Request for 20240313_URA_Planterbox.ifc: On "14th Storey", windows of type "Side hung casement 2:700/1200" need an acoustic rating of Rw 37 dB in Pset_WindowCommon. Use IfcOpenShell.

First a look at what the model holds.

```python
import ifcopenshell
import ifcopenshell.util.element

model = ifcopenshell.open("20240313_URA_Planterbox.ifc")
print(model.schema)
storey = next(s for s in model.by_type("IfcBuildingStorey") if s.Name == "14th Storey")
windows = [e for e in ifcopenshell.util.element.get_decomposition(storey) if e.is_a("IfcWindow")]
seen = {}
for e in windows:
    element_type = ifcopenshell.util.element.get_type(e)
    key = (element_type.Name if element_type != e and element_type else None, ifcopenshell.util.element.get_pset(e, "Pset_WindowCommon", "AcousticRating"))
    seen[key] = seen.get(key, 0) + 1
for (name, value), count in sorted(seen.items(), key=str):
    print(count, "x", name, "|", value)
```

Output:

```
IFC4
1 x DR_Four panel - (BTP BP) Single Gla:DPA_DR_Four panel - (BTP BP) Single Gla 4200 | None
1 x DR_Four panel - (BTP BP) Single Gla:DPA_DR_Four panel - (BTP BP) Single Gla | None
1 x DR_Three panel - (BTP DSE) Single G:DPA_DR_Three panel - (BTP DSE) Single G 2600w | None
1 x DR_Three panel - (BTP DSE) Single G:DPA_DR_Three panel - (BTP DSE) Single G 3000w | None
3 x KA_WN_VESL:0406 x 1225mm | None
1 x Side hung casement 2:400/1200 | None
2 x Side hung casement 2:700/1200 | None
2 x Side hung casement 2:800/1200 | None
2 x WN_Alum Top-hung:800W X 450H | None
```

```python
import ifcopenshell
import ifcopenshell.api.pset
import ifcopenshell.util.element

model = ifcopenshell.open("20240313_URA_Planterbox.ifc")

storey = next(s for s in model.by_type("IfcBuildingStorey") if s.Name == "14th Storey")
windows = [e for e in ifcopenshell.util.element.get_decomposition(storey) if e.is_a("IfcWindow")]

count = 0
for e in windows:
    element_type = ifcopenshell.util.element.get_type(e)
    if element_type in (None, e) or element_type.Name != "Side hung casement 2:700/1200":
        continue
    # add_pset returns the element's existing set when there is one.
    pset = ifcopenshell.api.pset.add_pset(model, product=e, name="Pset_WindowCommon")
    ifcopenshell.api.pset.edit_pset(model, pset=pset, properties={"AcousticRating": "Rw 37 dB"})
    count += 1

print(count, "windows updated")

model.write("20240313_URA_Planterbox_rev.ifc")
```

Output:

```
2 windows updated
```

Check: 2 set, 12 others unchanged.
